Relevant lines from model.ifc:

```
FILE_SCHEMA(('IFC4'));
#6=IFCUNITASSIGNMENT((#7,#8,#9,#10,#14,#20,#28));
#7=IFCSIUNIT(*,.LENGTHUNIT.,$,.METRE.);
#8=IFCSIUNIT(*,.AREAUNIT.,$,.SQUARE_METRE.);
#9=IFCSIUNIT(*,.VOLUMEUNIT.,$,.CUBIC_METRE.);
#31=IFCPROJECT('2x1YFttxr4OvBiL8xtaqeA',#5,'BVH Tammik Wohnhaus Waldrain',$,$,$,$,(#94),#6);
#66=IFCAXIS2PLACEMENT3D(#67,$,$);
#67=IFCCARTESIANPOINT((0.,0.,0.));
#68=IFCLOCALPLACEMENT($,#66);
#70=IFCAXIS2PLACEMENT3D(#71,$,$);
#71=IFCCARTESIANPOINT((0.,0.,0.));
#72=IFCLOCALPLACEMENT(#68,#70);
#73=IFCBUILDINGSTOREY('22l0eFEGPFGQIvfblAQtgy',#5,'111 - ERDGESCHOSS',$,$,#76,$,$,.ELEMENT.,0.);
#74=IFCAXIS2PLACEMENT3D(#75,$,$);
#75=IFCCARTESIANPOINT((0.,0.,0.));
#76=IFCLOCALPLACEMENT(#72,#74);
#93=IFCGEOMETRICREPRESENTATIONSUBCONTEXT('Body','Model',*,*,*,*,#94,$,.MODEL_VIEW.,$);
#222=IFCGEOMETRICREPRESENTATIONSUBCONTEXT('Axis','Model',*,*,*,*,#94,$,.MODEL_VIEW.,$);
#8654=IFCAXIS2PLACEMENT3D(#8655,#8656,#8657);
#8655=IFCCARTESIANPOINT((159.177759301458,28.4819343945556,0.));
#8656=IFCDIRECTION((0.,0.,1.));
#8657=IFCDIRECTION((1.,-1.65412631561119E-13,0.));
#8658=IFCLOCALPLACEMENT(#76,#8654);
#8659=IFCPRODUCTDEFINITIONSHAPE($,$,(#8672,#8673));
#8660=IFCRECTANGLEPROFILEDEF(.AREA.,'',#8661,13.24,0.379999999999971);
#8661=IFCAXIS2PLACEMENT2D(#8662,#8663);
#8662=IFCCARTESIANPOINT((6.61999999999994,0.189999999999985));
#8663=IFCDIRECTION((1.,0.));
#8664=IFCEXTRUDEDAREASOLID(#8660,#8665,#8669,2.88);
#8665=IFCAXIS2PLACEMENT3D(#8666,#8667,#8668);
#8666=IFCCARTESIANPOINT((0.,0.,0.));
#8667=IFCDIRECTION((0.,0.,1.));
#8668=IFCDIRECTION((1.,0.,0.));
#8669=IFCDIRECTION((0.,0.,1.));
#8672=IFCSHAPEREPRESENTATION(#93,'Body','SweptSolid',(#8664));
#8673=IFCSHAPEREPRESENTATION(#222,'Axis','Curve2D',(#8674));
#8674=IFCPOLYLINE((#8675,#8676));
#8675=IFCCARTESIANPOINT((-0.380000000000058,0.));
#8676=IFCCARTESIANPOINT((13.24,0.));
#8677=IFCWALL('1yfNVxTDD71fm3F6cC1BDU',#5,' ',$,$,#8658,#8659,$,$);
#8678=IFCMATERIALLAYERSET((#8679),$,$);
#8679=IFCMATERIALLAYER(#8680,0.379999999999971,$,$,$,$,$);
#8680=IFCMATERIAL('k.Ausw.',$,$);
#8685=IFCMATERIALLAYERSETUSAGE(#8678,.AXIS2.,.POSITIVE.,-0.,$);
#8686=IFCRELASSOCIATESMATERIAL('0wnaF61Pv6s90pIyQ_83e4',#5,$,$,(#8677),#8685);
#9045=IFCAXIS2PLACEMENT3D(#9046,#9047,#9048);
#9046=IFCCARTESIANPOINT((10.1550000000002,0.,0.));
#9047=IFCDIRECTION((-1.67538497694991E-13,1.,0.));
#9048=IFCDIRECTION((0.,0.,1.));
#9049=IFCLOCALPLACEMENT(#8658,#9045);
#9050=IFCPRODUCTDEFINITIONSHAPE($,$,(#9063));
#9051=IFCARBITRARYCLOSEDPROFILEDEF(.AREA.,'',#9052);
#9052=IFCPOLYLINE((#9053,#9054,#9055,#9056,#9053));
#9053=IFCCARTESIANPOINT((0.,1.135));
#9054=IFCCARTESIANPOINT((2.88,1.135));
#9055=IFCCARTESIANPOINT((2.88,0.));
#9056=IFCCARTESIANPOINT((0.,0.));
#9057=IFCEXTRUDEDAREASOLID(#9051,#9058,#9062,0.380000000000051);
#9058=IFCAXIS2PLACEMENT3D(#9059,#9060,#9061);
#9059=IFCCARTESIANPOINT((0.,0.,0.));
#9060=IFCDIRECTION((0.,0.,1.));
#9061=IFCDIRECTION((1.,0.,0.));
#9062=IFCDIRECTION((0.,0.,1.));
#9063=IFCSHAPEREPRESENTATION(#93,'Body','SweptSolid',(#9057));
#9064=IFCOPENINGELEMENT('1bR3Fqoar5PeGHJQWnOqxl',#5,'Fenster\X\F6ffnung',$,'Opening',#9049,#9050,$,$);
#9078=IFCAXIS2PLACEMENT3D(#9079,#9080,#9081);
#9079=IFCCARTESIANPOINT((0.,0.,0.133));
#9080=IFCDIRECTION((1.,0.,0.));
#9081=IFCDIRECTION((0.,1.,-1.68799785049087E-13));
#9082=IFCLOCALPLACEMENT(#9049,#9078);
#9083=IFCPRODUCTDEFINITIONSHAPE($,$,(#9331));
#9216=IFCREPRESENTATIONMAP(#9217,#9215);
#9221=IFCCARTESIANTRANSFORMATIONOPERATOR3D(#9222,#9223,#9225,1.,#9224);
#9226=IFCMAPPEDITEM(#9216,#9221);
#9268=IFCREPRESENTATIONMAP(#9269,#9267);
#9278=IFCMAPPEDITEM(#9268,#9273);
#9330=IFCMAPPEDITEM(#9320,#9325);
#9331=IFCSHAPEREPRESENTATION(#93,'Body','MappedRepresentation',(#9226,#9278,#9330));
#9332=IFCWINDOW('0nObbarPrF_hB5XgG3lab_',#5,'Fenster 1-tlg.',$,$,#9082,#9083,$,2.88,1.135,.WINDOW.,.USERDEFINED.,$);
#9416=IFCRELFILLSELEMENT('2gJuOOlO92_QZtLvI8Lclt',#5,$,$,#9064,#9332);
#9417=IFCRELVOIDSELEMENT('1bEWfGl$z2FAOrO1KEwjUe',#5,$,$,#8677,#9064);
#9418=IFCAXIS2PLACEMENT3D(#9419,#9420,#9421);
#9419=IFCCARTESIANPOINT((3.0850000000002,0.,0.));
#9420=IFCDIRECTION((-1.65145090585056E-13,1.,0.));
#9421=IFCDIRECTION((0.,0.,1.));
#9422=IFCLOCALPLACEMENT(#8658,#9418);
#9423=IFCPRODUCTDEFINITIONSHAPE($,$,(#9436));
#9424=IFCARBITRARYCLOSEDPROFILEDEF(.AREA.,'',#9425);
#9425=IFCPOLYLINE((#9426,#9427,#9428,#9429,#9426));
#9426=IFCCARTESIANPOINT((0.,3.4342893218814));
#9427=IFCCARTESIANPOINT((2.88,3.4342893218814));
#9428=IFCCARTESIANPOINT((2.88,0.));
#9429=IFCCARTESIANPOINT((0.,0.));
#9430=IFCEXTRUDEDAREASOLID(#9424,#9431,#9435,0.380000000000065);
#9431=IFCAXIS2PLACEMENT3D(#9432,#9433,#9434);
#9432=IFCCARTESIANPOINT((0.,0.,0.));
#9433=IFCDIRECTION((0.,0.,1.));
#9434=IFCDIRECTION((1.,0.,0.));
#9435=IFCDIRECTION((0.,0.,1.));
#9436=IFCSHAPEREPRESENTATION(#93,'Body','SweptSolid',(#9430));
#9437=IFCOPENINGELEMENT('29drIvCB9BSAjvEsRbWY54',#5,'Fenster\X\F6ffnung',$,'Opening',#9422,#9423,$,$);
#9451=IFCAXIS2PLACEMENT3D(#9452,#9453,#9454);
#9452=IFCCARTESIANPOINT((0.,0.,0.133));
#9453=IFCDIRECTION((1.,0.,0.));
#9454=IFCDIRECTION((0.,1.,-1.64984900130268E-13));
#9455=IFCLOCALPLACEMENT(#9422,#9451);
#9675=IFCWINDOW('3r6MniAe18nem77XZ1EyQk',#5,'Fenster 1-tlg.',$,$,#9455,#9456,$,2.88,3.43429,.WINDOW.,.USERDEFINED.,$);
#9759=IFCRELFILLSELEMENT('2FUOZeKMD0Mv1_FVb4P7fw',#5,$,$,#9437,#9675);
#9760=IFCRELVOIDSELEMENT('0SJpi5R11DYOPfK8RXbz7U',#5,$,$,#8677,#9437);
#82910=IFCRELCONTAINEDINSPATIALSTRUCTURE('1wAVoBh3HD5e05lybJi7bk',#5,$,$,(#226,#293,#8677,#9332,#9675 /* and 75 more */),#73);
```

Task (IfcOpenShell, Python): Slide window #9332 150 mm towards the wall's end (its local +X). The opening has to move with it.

```python
import ifcopenshell
import ifcopenshell.api.geometry
import ifcopenshell.util.placement
import ifcopenshell.util.unit

model = ifcopenshell.open("model.ifc")
unit_scale = ifcopenshell.util.unit.calculate_unit_scale(model)

window = model.by_guid("0nObbarPrF_hB5XgG3lab_")
opening = window.FillsVoids[0].RelatingOpeningElement
wall = opening.VoidsElements[0].RelatingBuildingElement

wall_matrix = ifcopenshell.util.placement.get_local_placement(wall.ObjectPlacement)
shift = wall_matrix[:3, 0] * 0.15 / unit_scale
before = ifcopenshell.util.placement.get_local_placement(window.ObjectPlacement)[:3, 3].copy()

# The window is placed relative to its opening, so it follows when the opening moves.
matrix = ifcopenshell.util.placement.get_local_placement(opening.ObjectPlacement)
matrix[:3, 3] += shift
ifcopenshell.api.geometry.edit_object_placement(
    model, product=opening, matrix=matrix, is_si=False, should_transform_children=True
)

after = ifcopenshell.util.placement.get_local_placement(window.ObjectPlacement)[:3, 3]
print("window moved by", (after - before).round(3) + 0.0)

model.write("model-out.ifc")
```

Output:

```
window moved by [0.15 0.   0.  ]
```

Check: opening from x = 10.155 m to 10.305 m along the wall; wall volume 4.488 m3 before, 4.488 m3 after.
